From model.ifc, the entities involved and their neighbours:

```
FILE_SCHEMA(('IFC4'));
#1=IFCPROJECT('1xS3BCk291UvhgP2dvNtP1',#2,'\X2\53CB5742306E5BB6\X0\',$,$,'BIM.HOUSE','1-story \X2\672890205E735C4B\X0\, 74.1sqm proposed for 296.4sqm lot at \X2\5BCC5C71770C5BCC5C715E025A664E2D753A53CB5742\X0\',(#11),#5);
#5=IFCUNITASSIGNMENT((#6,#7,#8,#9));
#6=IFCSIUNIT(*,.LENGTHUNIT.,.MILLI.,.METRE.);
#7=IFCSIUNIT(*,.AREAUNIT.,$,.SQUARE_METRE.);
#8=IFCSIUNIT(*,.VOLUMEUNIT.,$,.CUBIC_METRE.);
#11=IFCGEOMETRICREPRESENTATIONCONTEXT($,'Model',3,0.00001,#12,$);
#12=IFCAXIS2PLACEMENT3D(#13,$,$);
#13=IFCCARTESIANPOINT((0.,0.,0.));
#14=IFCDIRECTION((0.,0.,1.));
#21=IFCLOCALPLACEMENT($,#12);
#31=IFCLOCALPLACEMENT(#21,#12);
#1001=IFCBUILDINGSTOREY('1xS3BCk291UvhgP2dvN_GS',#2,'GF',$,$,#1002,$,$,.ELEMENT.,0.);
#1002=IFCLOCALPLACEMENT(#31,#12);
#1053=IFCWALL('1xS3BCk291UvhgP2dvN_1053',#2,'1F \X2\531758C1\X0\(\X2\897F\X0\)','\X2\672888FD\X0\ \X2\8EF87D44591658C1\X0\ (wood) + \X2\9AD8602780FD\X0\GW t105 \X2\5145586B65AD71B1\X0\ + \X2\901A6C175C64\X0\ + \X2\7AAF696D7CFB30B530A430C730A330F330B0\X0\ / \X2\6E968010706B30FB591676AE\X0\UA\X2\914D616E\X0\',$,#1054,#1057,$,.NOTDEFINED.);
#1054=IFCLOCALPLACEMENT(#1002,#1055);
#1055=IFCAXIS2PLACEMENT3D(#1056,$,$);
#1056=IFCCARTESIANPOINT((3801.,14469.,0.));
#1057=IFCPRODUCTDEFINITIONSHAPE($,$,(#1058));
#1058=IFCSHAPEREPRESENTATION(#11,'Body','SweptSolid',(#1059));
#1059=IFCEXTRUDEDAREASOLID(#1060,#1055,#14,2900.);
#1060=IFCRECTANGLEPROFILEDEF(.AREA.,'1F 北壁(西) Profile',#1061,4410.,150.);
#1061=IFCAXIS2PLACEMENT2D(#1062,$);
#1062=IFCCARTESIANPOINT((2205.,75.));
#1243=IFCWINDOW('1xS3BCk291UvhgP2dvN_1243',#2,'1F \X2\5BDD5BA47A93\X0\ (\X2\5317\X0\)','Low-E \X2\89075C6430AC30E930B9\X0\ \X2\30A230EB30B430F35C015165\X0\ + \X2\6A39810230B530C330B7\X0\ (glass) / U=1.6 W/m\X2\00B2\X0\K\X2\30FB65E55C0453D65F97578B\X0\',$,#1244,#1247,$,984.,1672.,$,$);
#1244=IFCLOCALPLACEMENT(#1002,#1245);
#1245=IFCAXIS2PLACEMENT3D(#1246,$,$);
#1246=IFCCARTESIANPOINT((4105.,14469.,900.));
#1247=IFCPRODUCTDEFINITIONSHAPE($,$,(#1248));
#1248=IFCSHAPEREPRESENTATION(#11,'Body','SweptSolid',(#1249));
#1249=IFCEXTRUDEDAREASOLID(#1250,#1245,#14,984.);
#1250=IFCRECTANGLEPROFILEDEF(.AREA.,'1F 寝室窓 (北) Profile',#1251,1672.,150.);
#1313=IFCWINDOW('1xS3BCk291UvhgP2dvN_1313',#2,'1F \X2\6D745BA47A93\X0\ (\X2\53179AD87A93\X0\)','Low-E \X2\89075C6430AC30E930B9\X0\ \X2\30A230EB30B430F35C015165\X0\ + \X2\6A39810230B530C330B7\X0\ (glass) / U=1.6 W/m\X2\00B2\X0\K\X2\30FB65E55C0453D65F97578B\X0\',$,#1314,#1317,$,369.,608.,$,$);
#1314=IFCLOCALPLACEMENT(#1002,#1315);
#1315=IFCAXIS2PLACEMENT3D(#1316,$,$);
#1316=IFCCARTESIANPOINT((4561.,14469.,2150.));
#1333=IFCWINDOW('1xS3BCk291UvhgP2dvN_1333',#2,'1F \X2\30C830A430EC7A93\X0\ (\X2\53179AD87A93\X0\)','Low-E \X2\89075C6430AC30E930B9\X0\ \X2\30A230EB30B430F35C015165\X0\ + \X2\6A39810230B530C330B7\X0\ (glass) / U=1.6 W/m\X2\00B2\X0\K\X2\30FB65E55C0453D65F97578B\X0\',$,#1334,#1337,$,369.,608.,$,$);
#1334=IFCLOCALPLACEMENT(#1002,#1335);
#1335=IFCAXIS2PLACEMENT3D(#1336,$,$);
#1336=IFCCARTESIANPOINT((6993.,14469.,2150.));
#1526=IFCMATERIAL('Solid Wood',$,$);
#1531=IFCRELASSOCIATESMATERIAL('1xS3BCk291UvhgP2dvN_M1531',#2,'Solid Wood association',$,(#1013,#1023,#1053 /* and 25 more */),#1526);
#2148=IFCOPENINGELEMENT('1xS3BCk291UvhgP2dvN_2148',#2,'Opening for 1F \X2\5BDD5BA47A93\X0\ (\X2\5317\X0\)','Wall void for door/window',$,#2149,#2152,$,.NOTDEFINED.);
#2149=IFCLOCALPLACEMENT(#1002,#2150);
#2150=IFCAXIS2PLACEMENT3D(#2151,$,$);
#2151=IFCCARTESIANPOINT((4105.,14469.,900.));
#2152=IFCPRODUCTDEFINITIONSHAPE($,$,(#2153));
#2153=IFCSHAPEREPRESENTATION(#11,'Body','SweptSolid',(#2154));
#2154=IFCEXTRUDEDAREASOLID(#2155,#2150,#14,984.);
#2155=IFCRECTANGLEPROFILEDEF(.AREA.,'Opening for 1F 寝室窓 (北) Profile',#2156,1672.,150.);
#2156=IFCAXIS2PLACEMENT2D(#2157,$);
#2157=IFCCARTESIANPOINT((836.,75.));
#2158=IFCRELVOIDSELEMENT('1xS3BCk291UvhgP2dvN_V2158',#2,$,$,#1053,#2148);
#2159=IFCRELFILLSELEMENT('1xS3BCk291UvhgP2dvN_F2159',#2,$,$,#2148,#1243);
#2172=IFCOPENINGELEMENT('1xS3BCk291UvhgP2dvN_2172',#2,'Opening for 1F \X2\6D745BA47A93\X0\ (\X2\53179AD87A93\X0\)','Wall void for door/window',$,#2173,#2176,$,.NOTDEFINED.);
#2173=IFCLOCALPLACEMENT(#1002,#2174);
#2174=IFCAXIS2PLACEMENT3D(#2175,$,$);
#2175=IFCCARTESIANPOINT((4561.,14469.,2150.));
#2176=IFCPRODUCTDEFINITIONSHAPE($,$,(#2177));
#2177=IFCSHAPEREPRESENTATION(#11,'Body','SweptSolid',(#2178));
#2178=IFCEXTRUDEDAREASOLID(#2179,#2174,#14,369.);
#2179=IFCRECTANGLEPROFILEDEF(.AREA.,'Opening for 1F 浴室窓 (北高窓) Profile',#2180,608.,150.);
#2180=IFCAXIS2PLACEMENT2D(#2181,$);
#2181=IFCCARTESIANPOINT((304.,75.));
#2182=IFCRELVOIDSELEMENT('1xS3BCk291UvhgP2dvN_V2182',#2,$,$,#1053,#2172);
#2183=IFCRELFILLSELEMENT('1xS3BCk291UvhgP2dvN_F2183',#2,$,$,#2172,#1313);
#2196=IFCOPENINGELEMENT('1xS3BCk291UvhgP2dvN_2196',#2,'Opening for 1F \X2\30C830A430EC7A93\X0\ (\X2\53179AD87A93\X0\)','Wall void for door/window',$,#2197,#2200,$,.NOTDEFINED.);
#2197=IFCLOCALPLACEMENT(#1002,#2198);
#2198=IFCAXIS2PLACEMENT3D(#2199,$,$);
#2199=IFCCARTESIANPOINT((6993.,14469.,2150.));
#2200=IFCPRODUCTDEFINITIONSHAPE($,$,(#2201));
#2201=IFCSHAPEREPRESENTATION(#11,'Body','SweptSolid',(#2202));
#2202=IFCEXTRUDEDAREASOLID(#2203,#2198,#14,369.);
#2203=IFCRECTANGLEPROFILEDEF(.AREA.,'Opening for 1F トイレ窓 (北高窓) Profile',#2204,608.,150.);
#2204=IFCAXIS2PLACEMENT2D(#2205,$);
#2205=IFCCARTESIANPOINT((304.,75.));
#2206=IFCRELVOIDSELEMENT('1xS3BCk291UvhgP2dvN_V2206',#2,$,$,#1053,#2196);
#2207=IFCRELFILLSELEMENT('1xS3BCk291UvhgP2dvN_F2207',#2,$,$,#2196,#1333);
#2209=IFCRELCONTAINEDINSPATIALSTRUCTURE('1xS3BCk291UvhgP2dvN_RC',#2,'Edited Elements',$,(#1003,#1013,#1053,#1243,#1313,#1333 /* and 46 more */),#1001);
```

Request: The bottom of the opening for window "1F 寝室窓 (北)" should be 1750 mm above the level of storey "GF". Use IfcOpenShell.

```python
import numpy as np
import ifcopenshell
import ifcopenshell.api.geometry
import ifcopenshell.geom
import ifcopenshell.util.element
import ifcopenshell.util.placement
import ifcopenshell.util.shape
import ifcopenshell.util.unit

model = ifcopenshell.open("model.ifc")
unit_scale = ifcopenshell.util.unit.calculate_unit_scale(model)

window = model.by_guid("1xS3BCk291UvhgP2dvN_1243")
opening = window.FillsVoids[0].RelatingOpeningElement
storey = ifcopenshell.util.element.get_container(window, ifc_class="IfcBuildingStorey")
level = ifcopenshell.util.placement.get_local_placement(storey.ObjectPlacement)[2, 3]

# The opening's origin need not be at the sill, so measure its lowest point.
shape = ifcopenshell.geom.create_shape(ifcopenshell.geom.settings(), opening)
bottom = ifcopenshell.util.shape.get_shape_bottom_elevation(shape, shape.geometry) / unit_scale
dz = level + 1.75 / unit_scale - bottom

shift = np.array([0.0, 0.0, dz])
# The window is not placed relative to its opening, so move both.
for product in (opening, window):
    matrix = ifcopenshell.util.placement.get_local_placement(product.ObjectPlacement)
    matrix[:3, 3] += shift
    ifcopenshell.api.geometry.edit_object_placement(model, product=product, matrix=matrix, is_si=False)

print(f"moved by {dz * unit_scale:+.3f} m")

model.write("model_rev.ifc")
```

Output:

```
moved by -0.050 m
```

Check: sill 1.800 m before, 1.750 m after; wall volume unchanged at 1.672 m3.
